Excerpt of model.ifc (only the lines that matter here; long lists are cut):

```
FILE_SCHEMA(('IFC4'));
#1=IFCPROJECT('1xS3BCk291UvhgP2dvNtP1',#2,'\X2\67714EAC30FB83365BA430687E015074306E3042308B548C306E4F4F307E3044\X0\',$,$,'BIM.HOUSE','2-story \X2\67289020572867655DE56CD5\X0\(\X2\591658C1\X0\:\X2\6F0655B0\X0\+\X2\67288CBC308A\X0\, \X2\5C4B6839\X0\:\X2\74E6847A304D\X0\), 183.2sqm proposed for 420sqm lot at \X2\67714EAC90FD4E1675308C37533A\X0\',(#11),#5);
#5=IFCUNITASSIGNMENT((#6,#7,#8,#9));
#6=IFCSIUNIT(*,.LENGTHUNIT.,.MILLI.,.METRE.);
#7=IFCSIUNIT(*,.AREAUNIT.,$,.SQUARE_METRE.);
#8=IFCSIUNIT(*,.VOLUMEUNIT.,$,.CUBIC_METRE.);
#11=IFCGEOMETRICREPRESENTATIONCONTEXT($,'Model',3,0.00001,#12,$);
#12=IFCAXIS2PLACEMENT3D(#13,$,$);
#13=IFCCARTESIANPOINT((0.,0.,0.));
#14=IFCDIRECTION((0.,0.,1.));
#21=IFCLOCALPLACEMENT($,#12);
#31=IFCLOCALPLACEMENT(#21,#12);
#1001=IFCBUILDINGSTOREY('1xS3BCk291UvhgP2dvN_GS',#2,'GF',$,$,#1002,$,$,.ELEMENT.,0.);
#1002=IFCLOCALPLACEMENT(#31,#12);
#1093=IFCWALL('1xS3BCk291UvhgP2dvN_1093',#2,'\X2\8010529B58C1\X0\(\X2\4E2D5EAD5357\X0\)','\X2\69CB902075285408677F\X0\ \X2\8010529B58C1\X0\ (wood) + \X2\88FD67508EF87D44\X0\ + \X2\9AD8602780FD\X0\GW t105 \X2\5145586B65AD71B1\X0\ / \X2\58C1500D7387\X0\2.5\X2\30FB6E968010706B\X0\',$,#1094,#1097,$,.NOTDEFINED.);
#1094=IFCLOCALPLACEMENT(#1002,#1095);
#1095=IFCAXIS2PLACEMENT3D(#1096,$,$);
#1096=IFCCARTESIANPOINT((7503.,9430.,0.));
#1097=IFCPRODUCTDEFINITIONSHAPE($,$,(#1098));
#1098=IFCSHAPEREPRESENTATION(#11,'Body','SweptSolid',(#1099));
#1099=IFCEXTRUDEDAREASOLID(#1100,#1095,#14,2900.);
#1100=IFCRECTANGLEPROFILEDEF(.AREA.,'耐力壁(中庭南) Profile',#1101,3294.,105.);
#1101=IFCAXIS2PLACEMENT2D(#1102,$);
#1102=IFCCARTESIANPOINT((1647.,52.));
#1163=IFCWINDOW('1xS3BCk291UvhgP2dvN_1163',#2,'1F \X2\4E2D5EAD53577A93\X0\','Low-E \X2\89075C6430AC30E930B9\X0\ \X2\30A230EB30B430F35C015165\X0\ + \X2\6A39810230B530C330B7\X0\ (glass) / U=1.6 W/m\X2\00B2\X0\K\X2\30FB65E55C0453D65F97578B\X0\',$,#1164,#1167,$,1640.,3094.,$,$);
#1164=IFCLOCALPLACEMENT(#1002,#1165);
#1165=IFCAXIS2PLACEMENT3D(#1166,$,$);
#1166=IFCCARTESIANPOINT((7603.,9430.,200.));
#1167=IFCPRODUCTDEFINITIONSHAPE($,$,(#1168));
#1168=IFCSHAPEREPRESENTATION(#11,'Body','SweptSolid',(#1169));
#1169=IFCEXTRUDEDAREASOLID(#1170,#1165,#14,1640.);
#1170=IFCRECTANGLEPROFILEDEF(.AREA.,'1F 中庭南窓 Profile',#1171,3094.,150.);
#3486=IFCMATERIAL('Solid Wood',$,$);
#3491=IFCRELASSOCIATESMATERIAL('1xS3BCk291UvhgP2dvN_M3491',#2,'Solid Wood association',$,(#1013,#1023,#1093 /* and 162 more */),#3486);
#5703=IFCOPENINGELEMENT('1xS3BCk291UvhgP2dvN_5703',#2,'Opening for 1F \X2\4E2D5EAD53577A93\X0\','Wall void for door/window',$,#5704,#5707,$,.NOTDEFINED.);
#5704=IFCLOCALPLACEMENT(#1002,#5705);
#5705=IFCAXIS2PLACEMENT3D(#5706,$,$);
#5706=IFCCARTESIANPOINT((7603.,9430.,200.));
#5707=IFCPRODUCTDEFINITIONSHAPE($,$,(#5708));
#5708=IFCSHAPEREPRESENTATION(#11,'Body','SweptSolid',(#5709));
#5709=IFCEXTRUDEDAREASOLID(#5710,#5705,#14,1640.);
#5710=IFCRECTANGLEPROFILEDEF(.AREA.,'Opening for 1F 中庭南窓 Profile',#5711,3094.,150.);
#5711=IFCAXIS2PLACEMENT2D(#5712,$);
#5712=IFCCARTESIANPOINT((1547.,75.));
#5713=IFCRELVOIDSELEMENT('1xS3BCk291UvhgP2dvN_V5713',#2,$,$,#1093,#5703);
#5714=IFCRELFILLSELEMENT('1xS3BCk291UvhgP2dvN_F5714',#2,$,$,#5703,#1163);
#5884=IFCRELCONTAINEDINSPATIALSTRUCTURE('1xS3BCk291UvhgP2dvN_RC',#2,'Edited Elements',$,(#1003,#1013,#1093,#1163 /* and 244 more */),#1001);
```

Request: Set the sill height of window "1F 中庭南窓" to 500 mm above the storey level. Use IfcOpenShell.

```python
import numpy as np
import ifcopenshell
import ifcopenshell.api.geometry
import ifcopenshell.geom
import ifcopenshell.util.element
import ifcopenshell.util.placement
import ifcopenshell.util.shape
import ifcopenshell.util.unit

model = ifcopenshell.open("model.ifc")
unit_scale = ifcopenshell.util.unit.calculate_unit_scale(model)

window = model.by_guid("1xS3BCk291UvhgP2dvN_1163")
opening = window.FillsVoids[0].RelatingOpeningElement
storey = ifcopenshell.util.element.get_container(window, ifc_class="IfcBuildingStorey")
level = ifcopenshell.util.placement.get_local_placement(storey.ObjectPlacement)[2, 3]

# The opening's origin need not be at the sill, so measure its lowest point.
shape = ifcopenshell.geom.create_shape(ifcopenshell.geom.settings(), opening)
bottom = ifcopenshell.util.shape.get_shape_bottom_elevation(shape, shape.geometry) / unit_scale
dz = level + 0.5 / unit_scale - bottom

shift = np.array([0.0, 0.0, dz])
# The window is not placed relative to its opening, so move both.
for product in (opening, window):
    matrix = ifcopenshell.util.placement.get_local_placement(product.ObjectPlacement)
    matrix[:3, 3] += shift
    ifcopenshell.api.geometry.edit_object_placement(model, product=product, matrix=matrix, is_si=False)

print(f"moved by {dz * unit_scale:+.3f} m")

model.write("model_edited.ifc")
```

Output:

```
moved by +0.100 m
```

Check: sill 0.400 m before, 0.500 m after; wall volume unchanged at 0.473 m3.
